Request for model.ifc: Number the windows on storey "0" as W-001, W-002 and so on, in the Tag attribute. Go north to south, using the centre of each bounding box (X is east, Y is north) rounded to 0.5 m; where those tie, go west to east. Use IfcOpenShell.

First a look at what the model holds.

```python
import ifcopenshell
import ifcopenshell.util.element
import ifcopenshell.util.placement

model = ifcopenshell.open("model.ifc")
print(model.schema)
storey = next(s for s in model.by_type("IfcBuildingStorey") if s.Name == "0")
windows = [e for e in ifcopenshell.util.element.get_decomposition(storey) if e.is_a("IfcWindow")]
for e in sorted(windows, key=lambda e: e.id()):
    origin = ifcopenshell.util.placement.get_local_placement(e.ObjectPlacement)[:3, 3]
    print(e.id(), e.Tag, e.Name, origin.round(2) + 0.0, sep=" | ")
```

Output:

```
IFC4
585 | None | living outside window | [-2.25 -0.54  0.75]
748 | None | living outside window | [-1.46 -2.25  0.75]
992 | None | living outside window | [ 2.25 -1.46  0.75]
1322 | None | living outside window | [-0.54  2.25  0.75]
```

```python
import ifcopenshell
import ifcopenshell.geom
import ifcopenshell.util.element
import ifcopenshell.util.shape

model = ifcopenshell.open("model.ifc")
settings = ifcopenshell.geom.settings()
settings.set("use-world-coords", True)


def centre(element):
    shape = ifcopenshell.geom.create_shape(settings, element)
    return ifcopenshell.util.shape.get_bbox_centroid(shape.geometry)


storey = next(s for s in model.by_type("IfcBuildingStorey") if s.Name == "0")
windows = [e for e in ifcopenshell.util.element.get_decomposition(storey) if e.is_a("IfcWindow")]

# Insertion points can sit at a corner or the storey origin, so sort by the geometry (in metres).
centres = {e: centre(e) for e in windows}
windows.sort(key=lambda e: (-round(centres[e][1] / 0.5), centres[e][0]))

for i, e in enumerate(windows, start=1):
    number = f"W-0{i:02d}"
    e.Tag = number
    print(e.id(), number)

model.write("model_rev.ifc")
```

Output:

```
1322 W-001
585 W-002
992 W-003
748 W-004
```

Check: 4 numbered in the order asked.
